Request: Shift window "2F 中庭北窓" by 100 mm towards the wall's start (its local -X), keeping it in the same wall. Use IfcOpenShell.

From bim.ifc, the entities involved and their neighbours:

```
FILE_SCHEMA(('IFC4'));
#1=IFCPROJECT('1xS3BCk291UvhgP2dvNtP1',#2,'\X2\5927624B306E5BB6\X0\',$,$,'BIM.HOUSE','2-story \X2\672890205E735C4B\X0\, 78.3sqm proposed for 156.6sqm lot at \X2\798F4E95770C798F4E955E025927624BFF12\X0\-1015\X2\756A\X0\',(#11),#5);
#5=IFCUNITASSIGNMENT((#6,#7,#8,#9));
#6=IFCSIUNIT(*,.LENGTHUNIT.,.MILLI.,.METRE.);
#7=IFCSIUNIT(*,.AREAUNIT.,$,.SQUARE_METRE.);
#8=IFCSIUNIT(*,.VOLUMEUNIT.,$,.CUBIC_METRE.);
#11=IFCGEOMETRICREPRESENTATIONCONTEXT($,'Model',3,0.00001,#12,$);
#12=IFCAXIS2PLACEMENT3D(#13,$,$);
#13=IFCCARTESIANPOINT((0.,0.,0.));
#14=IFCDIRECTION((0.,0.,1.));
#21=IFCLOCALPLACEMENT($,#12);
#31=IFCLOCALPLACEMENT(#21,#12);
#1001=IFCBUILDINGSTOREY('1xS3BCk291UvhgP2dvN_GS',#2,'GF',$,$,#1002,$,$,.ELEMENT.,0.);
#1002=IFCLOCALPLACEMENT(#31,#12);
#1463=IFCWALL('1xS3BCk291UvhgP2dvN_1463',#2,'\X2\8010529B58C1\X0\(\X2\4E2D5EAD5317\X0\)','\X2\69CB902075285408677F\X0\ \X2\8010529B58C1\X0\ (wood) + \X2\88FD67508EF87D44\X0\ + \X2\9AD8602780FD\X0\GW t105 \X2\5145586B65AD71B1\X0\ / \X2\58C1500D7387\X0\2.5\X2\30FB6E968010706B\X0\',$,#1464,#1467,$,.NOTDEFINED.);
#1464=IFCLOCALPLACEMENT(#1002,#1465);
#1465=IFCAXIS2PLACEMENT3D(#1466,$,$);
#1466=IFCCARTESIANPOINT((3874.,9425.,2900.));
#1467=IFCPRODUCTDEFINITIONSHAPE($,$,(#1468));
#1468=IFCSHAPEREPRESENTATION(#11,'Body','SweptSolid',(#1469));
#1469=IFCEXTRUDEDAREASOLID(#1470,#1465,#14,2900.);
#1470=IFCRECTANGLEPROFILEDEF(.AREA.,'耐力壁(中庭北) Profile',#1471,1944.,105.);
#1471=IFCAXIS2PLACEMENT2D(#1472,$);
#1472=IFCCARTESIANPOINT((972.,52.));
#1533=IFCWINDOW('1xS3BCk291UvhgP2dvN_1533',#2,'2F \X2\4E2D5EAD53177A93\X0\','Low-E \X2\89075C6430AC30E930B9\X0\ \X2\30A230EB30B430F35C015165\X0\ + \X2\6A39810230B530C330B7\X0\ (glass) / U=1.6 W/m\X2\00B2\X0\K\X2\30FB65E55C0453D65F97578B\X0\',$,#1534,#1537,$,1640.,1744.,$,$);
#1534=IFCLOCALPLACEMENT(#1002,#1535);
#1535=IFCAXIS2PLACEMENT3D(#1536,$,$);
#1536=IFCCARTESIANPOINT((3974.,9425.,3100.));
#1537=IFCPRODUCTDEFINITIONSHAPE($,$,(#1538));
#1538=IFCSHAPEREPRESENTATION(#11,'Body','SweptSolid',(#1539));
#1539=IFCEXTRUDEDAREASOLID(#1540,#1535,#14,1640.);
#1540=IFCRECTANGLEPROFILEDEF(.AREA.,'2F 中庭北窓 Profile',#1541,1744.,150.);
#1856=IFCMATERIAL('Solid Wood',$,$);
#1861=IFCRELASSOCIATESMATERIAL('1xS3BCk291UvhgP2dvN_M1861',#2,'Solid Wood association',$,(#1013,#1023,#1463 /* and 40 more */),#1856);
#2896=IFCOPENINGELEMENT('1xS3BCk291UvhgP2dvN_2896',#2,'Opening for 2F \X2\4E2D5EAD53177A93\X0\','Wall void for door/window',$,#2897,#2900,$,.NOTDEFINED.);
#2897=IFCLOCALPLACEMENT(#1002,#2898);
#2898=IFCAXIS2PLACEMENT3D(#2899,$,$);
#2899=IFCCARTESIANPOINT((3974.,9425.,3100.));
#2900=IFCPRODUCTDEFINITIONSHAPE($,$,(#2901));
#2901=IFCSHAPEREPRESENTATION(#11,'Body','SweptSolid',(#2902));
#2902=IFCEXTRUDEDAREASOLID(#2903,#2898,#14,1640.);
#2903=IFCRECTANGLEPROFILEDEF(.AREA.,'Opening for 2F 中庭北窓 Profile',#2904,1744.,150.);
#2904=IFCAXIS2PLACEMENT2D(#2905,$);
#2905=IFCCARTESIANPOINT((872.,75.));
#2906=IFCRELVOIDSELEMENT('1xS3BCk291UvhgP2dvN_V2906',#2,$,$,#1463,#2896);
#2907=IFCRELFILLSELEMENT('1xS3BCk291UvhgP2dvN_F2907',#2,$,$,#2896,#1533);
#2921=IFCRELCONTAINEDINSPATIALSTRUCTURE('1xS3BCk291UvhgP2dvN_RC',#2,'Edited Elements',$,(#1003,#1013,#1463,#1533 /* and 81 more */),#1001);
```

```python
import ifcopenshell
import ifcopenshell.api.geometry
import ifcopenshell.util.placement

model = ifcopenshell.open("bim.ifc")

window = model.by_guid("1xS3BCk291UvhgP2dvN_1533")
opening = window.FillsVoids[0].RelatingOpeningElement
wall = opening.VoidsElements[0].RelatingBuildingElement

wall_matrix = ifcopenshell.util.placement.get_local_placement(wall.ObjectPlacement)
shift = wall_matrix[:3, 0] * -100.0
before = ifcopenshell.util.placement.get_local_placement(window.ObjectPlacement)[:3, 3].copy()

# The window is not placed relative to its opening, so move both.
for product in (opening, window):
    matrix = ifcopenshell.util.placement.get_local_placement(product.ObjectPlacement)
    matrix[:3, 3] += shift
    ifcopenshell.api.geometry.edit_object_placement(model, product=product, matrix=matrix, is_si=False)

after = ifcopenshell.util.placement.get_local_placement(window.ObjectPlacement)[:3, 3]
print("window moved by", (after - before).round(3) + 0.0)

model.write("bim-out.ifc")
```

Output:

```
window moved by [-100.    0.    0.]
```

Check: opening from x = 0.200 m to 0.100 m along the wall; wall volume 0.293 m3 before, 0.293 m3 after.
